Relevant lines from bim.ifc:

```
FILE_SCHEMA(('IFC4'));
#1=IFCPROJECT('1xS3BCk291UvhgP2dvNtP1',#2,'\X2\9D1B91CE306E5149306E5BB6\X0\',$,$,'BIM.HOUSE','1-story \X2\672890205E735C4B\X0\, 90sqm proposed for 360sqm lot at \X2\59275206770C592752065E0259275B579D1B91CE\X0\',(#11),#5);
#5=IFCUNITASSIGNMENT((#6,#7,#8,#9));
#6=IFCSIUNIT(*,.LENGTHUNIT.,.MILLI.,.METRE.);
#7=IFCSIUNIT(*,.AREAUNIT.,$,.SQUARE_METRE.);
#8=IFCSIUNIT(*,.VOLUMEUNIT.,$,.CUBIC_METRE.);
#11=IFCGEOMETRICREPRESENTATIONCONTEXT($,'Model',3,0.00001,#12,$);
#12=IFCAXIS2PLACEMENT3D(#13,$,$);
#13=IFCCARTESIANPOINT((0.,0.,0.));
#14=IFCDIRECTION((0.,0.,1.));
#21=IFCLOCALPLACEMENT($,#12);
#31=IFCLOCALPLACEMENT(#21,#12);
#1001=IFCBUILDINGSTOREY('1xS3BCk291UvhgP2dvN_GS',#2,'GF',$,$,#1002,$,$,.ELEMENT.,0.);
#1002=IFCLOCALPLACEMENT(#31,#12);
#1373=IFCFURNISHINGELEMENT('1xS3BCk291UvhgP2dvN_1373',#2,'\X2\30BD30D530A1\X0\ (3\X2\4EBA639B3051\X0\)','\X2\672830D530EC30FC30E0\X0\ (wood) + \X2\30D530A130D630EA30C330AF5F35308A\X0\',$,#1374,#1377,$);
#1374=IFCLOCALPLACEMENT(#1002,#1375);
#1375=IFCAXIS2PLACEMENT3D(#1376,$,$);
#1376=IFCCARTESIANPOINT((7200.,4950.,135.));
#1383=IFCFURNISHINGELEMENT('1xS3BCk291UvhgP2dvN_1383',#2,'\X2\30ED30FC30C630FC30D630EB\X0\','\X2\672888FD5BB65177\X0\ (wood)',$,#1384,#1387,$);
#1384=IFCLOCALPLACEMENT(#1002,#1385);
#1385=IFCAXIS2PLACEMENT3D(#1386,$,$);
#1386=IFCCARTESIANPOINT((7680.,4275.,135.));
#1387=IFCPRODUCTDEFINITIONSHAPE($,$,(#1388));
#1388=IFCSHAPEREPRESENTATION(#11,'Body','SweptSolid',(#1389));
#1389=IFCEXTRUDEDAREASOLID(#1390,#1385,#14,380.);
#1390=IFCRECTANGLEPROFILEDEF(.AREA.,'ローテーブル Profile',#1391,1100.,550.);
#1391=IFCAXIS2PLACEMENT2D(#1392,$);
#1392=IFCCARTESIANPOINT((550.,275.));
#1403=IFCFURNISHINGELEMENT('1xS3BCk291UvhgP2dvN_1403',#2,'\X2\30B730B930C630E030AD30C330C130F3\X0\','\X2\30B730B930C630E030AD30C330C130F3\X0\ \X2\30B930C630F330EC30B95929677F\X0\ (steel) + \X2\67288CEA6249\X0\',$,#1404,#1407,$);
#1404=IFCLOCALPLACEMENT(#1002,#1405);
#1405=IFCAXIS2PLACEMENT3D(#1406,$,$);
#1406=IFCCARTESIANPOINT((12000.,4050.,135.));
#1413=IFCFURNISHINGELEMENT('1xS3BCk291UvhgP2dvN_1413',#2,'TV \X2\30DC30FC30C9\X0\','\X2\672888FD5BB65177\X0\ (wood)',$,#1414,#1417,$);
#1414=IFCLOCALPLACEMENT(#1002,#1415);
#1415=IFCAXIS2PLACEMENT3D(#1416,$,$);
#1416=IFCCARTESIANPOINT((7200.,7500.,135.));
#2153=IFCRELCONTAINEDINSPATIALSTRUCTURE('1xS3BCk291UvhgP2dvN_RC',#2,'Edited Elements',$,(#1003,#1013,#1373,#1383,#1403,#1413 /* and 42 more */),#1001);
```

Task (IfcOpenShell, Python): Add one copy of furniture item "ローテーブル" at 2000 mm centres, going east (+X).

```python
import numpy as np
import ifcopenshell
import ifcopenshell.api.geometry
import ifcopenshell.api.root
import ifcopenshell.util.element
import ifcopenshell.util.placement

model = ifcopenshell.open("bim.ifc")


def reuse_history(source, copy):
    """copy_class also copies each property set's owner history, people and application; keep the originals."""
    for rel in copy.IsDefinedBy:
        if rel.is_a("IfcRelDefinesByProperties") and (history := rel.RelatingPropertyDefinition.OwnerHistory):
            rel.RelatingPropertyDefinition.OwnerHistory = source.OwnerHistory
            ifcopenshell.util.element.remove_deep2(model, history)


source = model.by_guid("1xS3BCk291UvhgP2dvN_1383")
base = ifcopenshell.util.placement.get_local_placement(source.ObjectPlacement)
step = np.array([1.0, 0.0, 0.0]) * 2000.0

for i in range(1, 2):
    copy = ifcopenshell.api.root.copy_class(model, product=source)
    copy.Representation = ifcopenshell.util.element.copy_deep(
        model, source.Representation, exclude=["IfcGeometricRepresentationContext", "IfcRepresentationMap"]
    )
    reuse_history(source, copy)
    matrix = base.copy()
    matrix[:3, 3] += i * step
    print("added at", matrix[:3, 3].round(3) + 0.0)
    ifcopenshell.api.geometry.edit_object_placement(model, product=copy, matrix=matrix, is_si=False)

model.write("bim_updated.ifc")
```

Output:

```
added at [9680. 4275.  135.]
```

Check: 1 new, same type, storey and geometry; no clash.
